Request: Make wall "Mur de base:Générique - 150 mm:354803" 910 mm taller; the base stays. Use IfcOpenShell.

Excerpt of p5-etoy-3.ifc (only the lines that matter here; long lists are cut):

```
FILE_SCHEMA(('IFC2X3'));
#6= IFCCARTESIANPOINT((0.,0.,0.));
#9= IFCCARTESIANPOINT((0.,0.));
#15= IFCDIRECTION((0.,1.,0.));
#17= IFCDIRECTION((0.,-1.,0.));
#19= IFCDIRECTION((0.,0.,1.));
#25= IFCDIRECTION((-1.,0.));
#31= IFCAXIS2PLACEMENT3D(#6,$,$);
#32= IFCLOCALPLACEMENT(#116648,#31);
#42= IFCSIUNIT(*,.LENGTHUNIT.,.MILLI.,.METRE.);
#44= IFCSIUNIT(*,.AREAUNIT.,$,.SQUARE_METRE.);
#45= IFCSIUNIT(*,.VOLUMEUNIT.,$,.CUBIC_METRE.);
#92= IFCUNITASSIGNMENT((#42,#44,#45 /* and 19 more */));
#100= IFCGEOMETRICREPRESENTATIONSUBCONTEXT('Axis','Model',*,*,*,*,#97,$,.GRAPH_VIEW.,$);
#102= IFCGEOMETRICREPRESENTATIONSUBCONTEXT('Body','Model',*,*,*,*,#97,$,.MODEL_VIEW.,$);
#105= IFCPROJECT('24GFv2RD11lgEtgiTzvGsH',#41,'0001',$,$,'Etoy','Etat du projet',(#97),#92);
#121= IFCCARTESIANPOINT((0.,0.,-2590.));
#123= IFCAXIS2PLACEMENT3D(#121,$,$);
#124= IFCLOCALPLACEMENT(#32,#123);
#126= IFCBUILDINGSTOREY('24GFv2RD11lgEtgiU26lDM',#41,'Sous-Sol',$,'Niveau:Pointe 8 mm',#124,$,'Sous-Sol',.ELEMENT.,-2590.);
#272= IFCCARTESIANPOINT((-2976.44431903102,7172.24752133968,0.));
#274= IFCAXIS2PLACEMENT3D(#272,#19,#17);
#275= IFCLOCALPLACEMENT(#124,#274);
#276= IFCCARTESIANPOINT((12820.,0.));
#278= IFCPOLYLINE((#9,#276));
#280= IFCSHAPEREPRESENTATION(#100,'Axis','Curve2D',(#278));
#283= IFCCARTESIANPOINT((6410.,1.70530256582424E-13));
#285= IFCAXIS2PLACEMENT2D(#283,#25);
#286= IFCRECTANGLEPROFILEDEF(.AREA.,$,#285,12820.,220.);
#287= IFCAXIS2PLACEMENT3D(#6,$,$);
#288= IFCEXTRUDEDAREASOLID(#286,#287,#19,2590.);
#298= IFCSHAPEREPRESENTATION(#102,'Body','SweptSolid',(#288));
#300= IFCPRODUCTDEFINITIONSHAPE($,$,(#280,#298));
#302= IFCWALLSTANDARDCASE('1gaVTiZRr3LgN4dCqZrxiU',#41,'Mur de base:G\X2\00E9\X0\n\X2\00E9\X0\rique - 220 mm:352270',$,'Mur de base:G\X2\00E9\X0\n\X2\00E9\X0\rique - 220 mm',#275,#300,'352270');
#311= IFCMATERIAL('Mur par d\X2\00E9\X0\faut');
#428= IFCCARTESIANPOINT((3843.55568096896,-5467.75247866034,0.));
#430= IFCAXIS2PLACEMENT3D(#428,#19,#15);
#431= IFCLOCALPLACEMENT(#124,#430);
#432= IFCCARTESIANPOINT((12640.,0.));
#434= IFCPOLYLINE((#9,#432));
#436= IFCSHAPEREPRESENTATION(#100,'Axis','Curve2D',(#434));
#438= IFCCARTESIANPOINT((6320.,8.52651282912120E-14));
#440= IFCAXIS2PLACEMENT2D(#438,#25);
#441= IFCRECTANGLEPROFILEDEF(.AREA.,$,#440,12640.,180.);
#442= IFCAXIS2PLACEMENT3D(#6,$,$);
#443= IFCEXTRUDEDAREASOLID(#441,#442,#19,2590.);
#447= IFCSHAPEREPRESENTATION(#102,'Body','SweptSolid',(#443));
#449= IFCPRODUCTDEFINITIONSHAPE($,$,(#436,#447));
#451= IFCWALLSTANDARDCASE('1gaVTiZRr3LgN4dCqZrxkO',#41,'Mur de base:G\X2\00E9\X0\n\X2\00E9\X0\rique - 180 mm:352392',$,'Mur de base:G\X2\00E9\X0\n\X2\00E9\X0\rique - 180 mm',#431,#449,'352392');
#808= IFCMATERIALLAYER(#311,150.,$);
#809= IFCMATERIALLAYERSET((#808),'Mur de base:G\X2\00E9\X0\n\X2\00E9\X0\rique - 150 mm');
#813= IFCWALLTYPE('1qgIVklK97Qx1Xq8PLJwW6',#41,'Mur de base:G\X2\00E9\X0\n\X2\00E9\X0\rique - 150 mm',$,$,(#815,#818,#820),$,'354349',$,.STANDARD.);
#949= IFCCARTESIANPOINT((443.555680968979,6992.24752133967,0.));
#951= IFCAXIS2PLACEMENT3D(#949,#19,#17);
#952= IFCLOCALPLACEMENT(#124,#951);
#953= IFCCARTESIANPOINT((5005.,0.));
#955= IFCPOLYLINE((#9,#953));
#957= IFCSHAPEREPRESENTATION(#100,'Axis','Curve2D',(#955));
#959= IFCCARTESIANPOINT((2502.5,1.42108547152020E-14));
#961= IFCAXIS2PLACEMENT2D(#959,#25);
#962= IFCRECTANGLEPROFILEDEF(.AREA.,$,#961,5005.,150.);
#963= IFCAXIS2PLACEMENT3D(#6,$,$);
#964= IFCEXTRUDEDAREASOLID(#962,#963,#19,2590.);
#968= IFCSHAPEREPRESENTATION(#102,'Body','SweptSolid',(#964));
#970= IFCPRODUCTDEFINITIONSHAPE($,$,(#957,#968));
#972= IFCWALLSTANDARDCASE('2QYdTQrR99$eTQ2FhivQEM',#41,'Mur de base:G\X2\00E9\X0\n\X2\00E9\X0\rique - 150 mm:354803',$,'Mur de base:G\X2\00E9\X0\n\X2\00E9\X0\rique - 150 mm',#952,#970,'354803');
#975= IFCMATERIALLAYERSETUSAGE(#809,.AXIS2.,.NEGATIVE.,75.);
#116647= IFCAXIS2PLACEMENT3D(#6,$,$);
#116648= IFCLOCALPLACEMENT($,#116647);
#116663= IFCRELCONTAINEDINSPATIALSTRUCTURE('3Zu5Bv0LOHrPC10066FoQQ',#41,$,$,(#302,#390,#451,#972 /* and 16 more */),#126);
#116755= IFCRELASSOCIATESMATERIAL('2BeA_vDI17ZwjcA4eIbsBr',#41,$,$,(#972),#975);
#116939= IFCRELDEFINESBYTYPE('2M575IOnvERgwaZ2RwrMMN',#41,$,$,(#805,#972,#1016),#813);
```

```python
import ifcopenshell
import ifcopenshell.geom
import ifcopenshell.util.representation
import ifcopenshell.util.shape

model = ifcopenshell.open("p5-etoy-3.ifc")
settings = ifcopenshell.geom.settings()


def volume(element):
    """Net volume in cubic metres, openings subtracted."""
    shape = ifcopenshell.geom.create_shape(settings, element)
    return ifcopenshell.util.shape.get_volume(shape.geometry)


wall = model.by_id(972)
before = volume(wall)

body = ifcopenshell.util.representation.get_representation(wall, "Model", "Body")
solid = body.Items[0]
old_height = solid.Depth
solid.Depth += 910.0
after = volume(wall)

print(f"height {old_height:g} -> {solid.Depth:g}, volume {before:.3f} -> {after:.3f} m3")

model.write("p5-etoy-3_v2.ifc")
```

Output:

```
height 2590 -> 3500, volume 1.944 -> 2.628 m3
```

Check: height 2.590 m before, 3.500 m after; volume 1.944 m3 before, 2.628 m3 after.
